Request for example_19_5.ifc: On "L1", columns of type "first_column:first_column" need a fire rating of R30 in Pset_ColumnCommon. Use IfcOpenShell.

First a look at what the model holds.

```python
import ifcopenshell
import ifcopenshell.util.element

model = ifcopenshell.open("example_19_5.ifc")
print(model.schema)
storey = next(s for s in model.by_type("IfcBuildingStorey") if s.Name == "L1")
columns = [e for e in ifcopenshell.util.element.get_decomposition(storey) if e.is_a("IfcColumn")]
seen = {}
for e in columns:
    element_type = ifcopenshell.util.element.get_type(e)
    key = (element_type.Name if element_type != e and element_type else None, ifcopenshell.util.element.get_pset(e, "Pset_ColumnCommon", "FireRating"))
    seen[key] = seen.get(key, 0) + 1
for (name, value), count in sorted(seen.items(), key=str):
    print(count, "x", name, "|", value)
```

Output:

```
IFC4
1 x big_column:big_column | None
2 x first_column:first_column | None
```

```python
import ifcopenshell
import ifcopenshell.api.pset
import ifcopenshell.util.element

model = ifcopenshell.open("example_19_5.ifc")

storey = next(s for s in model.by_type("IfcBuildingStorey") if s.Name == "L1")
columns = [e for e in ifcopenshell.util.element.get_decomposition(storey) if e.is_a("IfcColumn")]

count = 0
for e in columns:
    element_type = ifcopenshell.util.element.get_type(e)
    if element_type in (None, e) or element_type.Name != "first_column:first_column":
        continue
    # add_pset returns the element's existing set when there is one.
    pset = ifcopenshell.api.pset.add_pset(model, product=e, name="Pset_ColumnCommon")
    ifcopenshell.api.pset.edit_pset(model, pset=pset, properties={"FireRating": "R30"})
    count += 1

print(count, "columns updated")

model.write("example_19_5_edited.ifc")
```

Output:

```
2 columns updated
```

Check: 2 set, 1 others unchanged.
